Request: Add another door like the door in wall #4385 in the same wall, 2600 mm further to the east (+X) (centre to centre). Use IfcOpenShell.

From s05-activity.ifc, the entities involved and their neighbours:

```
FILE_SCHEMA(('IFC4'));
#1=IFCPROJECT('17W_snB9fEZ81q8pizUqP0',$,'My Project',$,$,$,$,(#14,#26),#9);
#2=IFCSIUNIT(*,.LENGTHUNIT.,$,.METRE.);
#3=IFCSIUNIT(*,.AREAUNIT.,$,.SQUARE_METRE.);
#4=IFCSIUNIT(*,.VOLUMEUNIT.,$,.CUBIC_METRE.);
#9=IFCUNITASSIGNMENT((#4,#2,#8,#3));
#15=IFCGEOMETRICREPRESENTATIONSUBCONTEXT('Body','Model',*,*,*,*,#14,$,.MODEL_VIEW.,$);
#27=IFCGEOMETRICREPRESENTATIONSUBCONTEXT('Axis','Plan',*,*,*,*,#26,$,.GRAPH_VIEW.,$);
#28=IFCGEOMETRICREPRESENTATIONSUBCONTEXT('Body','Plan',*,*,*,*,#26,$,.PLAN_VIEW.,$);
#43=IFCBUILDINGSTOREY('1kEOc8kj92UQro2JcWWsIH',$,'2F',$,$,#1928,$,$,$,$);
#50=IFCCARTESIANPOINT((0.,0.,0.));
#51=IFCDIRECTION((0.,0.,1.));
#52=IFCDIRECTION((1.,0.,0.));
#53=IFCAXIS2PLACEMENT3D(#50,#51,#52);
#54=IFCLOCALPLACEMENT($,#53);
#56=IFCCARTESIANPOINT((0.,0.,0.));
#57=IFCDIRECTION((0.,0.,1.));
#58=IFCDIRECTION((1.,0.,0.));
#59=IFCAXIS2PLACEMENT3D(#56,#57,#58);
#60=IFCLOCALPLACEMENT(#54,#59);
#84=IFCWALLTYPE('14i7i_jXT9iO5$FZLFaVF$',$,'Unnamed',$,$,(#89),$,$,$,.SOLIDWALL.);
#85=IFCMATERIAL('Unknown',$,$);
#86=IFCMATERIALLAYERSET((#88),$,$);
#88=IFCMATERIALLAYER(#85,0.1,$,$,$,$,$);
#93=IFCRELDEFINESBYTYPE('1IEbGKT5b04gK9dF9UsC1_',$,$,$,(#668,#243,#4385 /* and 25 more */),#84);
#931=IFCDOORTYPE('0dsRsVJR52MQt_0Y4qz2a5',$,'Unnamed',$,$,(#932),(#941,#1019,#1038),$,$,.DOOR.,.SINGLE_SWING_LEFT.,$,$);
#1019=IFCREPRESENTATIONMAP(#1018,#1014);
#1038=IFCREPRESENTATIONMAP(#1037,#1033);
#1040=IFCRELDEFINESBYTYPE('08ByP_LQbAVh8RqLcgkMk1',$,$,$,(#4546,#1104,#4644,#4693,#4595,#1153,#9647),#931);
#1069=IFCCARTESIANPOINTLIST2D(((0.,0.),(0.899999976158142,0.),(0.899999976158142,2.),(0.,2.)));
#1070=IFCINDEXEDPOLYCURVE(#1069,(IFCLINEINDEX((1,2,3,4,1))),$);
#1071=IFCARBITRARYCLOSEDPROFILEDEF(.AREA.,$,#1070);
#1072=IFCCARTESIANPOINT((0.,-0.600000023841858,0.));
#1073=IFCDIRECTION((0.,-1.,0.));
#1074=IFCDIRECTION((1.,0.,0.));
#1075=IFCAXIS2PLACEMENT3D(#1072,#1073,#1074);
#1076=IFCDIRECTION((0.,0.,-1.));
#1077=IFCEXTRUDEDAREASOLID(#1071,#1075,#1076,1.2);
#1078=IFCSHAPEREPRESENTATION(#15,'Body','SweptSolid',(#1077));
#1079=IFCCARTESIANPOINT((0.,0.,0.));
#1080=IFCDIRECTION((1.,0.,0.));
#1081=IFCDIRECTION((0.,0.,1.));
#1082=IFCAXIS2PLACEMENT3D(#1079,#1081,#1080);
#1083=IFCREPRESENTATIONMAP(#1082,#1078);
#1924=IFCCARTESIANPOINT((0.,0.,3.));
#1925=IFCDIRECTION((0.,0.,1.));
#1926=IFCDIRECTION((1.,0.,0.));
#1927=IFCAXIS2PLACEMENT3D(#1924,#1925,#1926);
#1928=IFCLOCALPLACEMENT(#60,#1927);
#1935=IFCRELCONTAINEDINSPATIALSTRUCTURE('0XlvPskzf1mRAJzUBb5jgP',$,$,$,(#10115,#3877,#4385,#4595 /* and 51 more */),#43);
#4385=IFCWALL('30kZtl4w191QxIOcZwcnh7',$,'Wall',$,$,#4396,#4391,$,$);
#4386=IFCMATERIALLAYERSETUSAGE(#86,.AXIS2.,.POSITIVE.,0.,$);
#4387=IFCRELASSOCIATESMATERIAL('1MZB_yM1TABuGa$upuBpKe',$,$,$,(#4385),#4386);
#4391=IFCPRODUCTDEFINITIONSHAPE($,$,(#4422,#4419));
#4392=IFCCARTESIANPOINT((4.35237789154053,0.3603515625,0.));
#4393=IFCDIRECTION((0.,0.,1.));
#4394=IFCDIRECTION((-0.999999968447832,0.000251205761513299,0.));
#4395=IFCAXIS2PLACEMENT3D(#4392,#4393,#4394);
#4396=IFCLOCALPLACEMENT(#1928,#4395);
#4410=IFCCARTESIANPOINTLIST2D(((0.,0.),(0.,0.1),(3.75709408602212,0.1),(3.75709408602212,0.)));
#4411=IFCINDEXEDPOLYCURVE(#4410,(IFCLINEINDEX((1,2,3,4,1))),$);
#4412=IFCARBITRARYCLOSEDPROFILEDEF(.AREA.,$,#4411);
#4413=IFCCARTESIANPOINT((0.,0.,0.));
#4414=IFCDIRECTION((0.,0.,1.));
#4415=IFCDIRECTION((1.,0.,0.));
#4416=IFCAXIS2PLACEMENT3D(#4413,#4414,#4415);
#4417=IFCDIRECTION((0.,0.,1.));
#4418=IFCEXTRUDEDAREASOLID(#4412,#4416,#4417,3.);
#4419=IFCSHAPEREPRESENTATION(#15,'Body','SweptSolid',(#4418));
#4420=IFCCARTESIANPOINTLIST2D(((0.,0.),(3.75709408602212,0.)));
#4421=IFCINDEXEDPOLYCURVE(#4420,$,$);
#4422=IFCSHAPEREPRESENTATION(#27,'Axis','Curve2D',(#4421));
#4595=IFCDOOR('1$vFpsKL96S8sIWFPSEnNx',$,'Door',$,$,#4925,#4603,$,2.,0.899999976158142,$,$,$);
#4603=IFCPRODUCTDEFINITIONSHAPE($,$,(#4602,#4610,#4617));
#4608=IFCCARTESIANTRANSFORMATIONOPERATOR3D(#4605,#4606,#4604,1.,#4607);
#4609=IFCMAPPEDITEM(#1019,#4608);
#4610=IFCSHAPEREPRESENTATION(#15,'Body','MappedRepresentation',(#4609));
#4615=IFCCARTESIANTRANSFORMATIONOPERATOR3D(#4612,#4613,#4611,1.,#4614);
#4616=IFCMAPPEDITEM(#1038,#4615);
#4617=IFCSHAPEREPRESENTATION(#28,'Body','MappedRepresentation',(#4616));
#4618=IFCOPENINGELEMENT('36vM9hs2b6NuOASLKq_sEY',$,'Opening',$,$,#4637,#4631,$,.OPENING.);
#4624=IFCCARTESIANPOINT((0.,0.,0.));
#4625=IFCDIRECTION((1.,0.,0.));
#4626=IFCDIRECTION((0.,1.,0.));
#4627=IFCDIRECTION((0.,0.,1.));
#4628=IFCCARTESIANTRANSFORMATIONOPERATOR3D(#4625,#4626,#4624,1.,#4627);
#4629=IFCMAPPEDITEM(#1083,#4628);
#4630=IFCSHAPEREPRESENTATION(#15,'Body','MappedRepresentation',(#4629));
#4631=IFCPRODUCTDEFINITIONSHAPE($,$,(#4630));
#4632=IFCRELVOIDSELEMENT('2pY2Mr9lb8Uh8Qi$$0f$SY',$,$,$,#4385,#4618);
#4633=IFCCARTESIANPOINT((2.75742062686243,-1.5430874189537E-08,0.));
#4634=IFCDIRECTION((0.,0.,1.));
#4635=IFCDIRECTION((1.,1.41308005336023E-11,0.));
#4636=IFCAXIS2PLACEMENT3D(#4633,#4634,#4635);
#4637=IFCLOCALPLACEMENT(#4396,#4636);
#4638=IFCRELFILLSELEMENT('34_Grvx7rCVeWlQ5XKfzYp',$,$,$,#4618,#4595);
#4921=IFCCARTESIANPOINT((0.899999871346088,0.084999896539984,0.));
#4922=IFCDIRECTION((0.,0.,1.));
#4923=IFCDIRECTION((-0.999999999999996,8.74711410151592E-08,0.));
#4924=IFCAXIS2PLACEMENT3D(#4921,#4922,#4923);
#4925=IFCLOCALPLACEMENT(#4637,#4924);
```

```python
import ifcopenshell
import ifcopenshell.api.feature
import ifcopenshell.api.geometry
import ifcopenshell.api.root
import ifcopenshell.geom
import ifcopenshell.util.element
import ifcopenshell.util.placement
import ifcopenshell.util.shape
import ifcopenshell.util.unit

model = ifcopenshell.open("s05-activity.ifc")
unit_scale = ifcopenshell.util.unit.calculate_unit_scale(model)
settings = ifcopenshell.geom.settings()


def volume(element):
    """Net volume in cubic metres, openings subtracted."""
    shape = ifcopenshell.geom.create_shape(settings, element)
    return ifcopenshell.util.shape.get_volume(shape.geometry)


door = model.by_guid("1$vFpsKL96S8sIWFPSEnNx")
opening = door.FillsVoids[0].RelatingOpeningElement
wall = opening.VoidsElements[0].RelatingBuildingElement
before = volume(wall)
shift = ifcopenshell.util.placement.get_local_placement(wall.ObjectPlacement)[:3, 0] * -2.6 / unit_scale

# copy_class copies the void relationship, type, container and properties, but no geometry.
new_opening = ifcopenshell.api.root.copy_class(model, product=opening)
new_opening.Representation = ifcopenshell.util.element.copy_deep(
    model, opening.Representation, exclude=["IfcGeometricRepresentationContext", "IfcRepresentationMap"]
)
new_door = ifcopenshell.api.root.copy_class(model, product=door)
new_door.Representation = ifcopenshell.util.element.copy_deep(
    model, door.Representation, exclude=["IfcGeometricRepresentationContext", "IfcRepresentationMap"]
)
ifcopenshell.api.feature.add_filling(model, opening=new_opening, element=new_door)

for old, new in ((opening, new_opening), (door, new_door)):
    matrix = ifcopenshell.util.placement.get_local_placement(old.ObjectPlacement)
    matrix[:3, 3] += shift
    ifcopenshell.api.geometry.edit_object_placement(model, product=new, matrix=matrix, is_si=False)

after = volume(wall)

print(f"wall volume {before:.3f} -> {after:.3f} m3")

model.write("s05-activity_rev.ifc")
```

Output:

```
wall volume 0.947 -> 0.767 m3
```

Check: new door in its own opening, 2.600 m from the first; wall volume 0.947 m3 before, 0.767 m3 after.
